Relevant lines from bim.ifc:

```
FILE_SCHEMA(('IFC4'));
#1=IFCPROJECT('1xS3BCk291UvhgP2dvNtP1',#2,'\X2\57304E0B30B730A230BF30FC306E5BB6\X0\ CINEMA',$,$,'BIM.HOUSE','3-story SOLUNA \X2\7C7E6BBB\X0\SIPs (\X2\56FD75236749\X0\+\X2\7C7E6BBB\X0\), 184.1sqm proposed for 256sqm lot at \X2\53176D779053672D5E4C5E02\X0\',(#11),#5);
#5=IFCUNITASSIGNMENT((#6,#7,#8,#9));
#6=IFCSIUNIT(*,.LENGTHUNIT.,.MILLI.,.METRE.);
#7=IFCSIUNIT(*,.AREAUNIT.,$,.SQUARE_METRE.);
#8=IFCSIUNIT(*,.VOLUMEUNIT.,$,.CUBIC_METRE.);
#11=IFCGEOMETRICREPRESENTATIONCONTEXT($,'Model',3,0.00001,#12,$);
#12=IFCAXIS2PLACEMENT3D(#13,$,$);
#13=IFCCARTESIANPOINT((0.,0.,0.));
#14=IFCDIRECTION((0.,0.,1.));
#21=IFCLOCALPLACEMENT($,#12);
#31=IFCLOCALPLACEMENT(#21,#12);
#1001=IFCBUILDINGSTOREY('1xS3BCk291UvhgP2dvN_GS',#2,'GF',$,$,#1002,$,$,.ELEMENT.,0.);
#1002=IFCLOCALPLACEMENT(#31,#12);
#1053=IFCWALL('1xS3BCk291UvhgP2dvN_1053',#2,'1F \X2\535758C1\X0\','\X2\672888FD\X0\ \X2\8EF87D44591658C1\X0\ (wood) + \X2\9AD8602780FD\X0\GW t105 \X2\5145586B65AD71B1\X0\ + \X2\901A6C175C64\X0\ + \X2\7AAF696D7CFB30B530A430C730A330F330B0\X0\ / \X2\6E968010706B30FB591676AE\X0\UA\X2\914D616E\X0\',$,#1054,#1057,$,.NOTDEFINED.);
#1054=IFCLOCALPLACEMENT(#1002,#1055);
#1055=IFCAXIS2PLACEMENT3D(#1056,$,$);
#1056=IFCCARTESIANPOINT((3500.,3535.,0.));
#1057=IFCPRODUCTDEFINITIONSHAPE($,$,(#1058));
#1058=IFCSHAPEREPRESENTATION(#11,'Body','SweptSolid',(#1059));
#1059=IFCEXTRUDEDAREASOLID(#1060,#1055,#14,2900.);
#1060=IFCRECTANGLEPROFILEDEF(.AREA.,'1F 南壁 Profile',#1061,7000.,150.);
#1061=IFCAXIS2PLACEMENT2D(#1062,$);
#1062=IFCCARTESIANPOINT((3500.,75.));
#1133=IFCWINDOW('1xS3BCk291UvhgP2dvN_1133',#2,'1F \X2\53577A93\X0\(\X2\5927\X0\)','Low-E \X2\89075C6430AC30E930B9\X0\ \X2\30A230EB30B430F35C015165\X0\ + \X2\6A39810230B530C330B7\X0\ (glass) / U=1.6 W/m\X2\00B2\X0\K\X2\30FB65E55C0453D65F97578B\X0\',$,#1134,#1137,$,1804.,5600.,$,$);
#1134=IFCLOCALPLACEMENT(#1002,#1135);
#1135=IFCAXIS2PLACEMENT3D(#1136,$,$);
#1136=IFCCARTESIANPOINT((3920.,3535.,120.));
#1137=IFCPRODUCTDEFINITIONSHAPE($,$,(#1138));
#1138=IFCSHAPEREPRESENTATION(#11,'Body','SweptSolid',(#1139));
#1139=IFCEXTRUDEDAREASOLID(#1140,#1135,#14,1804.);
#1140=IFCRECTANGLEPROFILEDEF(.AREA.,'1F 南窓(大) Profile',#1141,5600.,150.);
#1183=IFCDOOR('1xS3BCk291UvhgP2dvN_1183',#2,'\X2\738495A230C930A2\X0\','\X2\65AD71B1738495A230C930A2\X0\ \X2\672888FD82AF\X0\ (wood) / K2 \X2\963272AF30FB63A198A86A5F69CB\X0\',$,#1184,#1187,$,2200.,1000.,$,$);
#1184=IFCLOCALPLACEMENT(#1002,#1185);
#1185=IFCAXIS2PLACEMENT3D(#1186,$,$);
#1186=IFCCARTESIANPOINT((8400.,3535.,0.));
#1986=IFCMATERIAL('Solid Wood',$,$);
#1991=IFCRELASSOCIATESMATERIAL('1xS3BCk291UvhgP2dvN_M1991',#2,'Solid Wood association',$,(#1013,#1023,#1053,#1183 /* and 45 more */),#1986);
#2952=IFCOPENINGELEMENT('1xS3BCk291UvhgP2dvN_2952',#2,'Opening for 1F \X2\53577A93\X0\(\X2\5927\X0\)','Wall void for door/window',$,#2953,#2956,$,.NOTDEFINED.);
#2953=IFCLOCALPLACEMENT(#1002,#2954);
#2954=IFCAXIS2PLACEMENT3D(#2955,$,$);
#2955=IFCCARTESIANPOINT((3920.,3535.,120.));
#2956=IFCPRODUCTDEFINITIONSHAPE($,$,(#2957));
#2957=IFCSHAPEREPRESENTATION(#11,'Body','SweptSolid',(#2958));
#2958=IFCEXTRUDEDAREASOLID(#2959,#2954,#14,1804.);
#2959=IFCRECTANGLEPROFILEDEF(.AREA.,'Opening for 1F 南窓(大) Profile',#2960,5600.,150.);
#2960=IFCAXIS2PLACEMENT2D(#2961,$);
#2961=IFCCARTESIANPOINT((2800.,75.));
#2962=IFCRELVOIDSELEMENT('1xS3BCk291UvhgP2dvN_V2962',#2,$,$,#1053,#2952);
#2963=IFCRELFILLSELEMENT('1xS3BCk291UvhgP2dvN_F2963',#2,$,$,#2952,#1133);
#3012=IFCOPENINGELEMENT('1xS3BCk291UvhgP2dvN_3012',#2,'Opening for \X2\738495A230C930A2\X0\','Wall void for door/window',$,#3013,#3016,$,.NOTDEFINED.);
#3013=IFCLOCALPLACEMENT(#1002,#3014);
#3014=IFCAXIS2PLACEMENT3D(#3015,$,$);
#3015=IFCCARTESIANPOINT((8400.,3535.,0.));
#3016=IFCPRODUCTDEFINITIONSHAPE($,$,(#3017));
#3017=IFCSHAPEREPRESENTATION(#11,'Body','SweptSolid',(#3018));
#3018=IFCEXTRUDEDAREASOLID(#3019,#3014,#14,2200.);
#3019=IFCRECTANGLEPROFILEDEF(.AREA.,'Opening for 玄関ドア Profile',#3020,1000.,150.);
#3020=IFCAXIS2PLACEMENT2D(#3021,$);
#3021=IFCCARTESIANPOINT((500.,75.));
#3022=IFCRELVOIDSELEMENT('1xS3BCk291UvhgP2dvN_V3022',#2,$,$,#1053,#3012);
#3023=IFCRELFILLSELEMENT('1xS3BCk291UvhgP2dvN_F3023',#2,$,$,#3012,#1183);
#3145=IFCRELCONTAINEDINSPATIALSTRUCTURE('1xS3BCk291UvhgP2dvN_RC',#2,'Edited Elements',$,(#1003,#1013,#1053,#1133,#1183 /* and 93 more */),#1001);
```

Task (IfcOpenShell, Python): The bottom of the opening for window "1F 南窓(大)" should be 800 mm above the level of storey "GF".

```python
import numpy as np
import ifcopenshell
import ifcopenshell.api.geometry
import ifcopenshell.geom
import ifcopenshell.util.element
import ifcopenshell.util.placement
import ifcopenshell.util.shape
import ifcopenshell.util.unit

model = ifcopenshell.open("bim.ifc")
unit_scale = ifcopenshell.util.unit.calculate_unit_scale(model)

window = model.by_guid("1xS3BCk291UvhgP2dvN_1133")
opening = window.FillsVoids[0].RelatingOpeningElement
storey = ifcopenshell.util.element.get_container(window, ifc_class="IfcBuildingStorey")
level = ifcopenshell.util.placement.get_local_placement(storey.ObjectPlacement)[2, 3]

# The opening's origin need not be at the sill, so measure its lowest point.
shape = ifcopenshell.geom.create_shape(ifcopenshell.geom.settings(), opening)
bottom = ifcopenshell.util.shape.get_shape_bottom_elevation(shape, shape.geometry) / unit_scale
dz = level + 800.0 - bottom

shift = np.array([0.0, 0.0, dz])
# The window is not placed relative to its opening, so move both.
for product in (opening, window):
    matrix = ifcopenshell.util.placement.get_local_placement(product.ObjectPlacement)
    matrix[:3, 3] += shift
    ifcopenshell.api.geometry.edit_object_placement(model, product=product, matrix=matrix, is_si=False)

print(f"moved by {dz * unit_scale:+.3f} m")

model.write("bim_rev.ifc")
```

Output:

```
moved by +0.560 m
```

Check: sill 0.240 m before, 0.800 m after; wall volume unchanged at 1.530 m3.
